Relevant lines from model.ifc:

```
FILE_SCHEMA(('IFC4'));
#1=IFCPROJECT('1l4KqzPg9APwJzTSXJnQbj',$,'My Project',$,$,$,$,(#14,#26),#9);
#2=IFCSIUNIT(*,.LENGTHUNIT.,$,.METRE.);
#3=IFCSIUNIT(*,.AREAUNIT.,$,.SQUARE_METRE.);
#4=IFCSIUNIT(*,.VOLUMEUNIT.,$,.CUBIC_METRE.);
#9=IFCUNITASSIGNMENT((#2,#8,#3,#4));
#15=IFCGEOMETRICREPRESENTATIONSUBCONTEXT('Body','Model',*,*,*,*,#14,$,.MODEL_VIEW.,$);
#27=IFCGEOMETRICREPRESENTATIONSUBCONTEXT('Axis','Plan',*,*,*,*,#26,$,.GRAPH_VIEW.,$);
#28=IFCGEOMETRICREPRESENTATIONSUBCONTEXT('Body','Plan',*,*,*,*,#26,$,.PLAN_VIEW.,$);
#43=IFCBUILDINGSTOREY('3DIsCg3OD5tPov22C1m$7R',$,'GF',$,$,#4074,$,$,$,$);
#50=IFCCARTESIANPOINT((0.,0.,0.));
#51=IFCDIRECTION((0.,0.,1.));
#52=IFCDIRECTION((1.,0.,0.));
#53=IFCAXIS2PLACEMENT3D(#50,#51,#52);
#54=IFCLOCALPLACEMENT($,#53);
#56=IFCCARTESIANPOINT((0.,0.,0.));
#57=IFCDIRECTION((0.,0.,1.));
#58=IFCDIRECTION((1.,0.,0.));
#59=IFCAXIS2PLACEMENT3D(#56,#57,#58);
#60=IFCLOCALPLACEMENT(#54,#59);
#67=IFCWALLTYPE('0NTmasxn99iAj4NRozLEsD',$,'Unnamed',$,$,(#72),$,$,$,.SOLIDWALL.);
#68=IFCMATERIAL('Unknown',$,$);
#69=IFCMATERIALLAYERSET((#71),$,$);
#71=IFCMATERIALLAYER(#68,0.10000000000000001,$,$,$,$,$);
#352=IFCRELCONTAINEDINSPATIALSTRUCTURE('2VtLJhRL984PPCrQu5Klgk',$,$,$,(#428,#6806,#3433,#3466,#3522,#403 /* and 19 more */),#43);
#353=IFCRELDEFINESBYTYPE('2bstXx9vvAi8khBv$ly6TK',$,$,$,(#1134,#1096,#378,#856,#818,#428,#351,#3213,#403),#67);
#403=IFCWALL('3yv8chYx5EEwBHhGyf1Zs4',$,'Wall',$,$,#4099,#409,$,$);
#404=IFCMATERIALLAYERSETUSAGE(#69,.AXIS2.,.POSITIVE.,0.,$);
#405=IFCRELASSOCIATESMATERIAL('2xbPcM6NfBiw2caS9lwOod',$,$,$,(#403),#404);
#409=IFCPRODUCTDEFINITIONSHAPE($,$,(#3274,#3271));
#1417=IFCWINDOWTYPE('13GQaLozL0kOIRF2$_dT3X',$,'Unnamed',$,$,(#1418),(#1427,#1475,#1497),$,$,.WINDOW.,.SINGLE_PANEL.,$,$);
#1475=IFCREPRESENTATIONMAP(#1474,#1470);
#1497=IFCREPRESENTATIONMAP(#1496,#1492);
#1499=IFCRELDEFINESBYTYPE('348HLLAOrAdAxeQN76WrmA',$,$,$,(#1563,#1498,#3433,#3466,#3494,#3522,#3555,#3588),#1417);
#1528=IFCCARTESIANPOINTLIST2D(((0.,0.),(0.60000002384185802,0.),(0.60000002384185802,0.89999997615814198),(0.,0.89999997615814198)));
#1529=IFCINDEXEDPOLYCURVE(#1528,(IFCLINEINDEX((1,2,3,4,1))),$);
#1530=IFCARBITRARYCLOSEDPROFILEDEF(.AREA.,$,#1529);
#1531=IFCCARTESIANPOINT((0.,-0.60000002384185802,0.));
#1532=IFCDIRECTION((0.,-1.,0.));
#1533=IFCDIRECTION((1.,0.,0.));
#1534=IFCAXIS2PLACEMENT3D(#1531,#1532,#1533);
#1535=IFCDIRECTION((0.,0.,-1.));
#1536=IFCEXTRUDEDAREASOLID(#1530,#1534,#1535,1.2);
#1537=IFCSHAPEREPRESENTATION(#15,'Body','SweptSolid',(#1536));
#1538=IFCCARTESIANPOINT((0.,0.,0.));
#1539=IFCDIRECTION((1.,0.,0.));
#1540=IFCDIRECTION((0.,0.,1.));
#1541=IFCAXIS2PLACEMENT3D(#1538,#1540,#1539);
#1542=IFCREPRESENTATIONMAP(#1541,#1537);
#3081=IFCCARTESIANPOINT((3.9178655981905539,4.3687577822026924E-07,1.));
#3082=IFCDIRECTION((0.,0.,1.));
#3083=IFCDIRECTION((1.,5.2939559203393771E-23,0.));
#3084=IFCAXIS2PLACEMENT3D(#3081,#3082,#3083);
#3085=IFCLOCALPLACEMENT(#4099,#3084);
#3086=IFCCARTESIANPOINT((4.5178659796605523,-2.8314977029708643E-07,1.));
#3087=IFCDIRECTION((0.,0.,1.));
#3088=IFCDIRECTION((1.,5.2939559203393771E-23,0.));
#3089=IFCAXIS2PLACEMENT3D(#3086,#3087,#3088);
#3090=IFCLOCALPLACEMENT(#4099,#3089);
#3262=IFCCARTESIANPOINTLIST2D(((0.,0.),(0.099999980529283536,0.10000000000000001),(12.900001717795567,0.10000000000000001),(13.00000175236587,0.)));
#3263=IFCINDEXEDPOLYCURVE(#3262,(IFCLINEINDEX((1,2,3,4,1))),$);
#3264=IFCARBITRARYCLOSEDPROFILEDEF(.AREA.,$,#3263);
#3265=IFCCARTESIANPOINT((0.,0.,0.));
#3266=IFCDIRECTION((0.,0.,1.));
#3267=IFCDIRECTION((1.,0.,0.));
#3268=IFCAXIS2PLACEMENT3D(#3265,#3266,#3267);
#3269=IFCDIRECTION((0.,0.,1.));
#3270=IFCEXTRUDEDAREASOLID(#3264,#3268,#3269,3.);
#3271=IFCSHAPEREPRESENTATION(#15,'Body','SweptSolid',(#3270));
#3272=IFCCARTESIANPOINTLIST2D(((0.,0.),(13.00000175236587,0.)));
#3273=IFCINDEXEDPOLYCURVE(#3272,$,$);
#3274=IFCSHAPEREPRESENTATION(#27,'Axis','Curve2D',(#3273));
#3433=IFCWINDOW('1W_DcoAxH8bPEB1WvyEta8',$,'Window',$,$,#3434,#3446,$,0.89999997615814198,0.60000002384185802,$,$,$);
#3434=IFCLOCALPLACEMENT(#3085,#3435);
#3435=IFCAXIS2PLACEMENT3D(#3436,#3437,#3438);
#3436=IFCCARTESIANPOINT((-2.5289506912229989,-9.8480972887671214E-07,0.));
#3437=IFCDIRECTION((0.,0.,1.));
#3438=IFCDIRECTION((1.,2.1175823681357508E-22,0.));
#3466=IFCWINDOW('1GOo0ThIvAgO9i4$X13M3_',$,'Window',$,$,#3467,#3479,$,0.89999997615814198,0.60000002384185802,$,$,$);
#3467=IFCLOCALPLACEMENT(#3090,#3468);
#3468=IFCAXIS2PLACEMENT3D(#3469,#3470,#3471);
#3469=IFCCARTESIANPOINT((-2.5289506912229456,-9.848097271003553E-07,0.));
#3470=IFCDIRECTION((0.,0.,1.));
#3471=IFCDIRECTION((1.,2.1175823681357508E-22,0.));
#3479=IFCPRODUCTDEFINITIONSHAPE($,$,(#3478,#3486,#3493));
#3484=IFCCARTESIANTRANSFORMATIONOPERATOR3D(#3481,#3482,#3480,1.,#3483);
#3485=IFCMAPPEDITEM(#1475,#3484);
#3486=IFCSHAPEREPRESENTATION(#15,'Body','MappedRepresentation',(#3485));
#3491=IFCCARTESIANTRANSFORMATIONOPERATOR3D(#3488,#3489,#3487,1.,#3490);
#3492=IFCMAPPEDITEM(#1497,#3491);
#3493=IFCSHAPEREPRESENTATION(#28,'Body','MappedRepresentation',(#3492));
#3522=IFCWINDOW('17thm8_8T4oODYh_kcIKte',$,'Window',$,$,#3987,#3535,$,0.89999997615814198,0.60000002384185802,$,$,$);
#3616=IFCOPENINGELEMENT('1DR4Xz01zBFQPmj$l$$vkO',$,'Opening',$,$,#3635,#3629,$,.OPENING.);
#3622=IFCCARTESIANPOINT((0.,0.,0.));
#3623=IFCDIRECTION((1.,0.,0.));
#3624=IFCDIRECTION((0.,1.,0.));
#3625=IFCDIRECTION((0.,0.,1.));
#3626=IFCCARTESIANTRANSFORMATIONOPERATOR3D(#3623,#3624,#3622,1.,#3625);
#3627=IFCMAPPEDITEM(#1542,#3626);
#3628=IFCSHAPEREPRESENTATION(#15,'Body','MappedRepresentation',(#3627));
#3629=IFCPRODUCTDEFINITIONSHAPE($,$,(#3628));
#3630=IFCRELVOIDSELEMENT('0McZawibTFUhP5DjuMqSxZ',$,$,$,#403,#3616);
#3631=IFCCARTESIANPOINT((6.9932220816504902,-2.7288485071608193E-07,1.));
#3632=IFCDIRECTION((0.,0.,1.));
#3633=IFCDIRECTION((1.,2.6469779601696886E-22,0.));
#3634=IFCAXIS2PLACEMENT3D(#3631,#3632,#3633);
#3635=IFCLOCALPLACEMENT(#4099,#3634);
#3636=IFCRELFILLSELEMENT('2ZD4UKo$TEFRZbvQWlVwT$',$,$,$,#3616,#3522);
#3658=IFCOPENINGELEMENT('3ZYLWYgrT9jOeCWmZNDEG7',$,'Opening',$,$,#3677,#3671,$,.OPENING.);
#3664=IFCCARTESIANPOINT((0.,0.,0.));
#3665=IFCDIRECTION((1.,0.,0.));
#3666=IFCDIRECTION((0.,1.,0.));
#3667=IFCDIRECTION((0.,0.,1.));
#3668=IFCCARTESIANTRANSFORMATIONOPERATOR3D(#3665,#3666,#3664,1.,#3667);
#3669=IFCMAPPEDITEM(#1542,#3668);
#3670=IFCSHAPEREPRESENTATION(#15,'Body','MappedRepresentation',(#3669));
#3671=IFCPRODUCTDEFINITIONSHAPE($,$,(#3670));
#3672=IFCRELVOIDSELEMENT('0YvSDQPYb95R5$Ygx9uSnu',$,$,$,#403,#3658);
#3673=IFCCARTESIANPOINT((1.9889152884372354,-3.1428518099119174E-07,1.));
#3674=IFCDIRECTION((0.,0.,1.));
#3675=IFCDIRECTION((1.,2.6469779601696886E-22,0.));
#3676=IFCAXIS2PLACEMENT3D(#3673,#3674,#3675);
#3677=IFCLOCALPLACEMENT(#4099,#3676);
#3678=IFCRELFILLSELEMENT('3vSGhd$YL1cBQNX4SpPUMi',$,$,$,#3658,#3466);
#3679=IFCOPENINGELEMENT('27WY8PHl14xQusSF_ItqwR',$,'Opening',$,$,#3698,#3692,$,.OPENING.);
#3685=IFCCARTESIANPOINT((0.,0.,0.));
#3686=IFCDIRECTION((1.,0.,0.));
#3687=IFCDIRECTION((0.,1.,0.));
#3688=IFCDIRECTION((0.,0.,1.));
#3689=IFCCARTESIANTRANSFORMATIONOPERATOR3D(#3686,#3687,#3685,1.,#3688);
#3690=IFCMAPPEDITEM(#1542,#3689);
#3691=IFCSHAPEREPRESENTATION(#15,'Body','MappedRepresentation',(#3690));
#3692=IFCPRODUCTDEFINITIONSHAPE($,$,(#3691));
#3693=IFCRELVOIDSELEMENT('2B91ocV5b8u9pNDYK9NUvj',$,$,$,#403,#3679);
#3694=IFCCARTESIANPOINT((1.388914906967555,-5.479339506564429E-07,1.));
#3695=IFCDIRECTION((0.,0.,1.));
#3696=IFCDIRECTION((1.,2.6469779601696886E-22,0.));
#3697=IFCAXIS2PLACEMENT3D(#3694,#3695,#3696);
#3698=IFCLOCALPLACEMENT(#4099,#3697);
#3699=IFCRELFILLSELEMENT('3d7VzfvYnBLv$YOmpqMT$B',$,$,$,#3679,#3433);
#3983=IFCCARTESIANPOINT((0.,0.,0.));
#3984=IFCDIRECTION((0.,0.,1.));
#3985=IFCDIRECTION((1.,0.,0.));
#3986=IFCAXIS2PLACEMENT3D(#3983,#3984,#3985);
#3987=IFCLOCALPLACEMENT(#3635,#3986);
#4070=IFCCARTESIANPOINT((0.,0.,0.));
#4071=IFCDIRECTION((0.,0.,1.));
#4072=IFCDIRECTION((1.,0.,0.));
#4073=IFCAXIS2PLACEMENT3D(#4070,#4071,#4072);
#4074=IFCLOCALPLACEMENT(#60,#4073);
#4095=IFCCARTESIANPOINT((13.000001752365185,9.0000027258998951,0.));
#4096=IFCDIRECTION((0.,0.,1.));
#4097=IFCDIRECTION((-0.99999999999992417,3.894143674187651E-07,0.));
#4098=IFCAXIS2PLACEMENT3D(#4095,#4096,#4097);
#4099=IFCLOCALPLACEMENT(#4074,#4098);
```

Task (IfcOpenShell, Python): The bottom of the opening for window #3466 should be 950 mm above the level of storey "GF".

```python
import numpy as np
import ifcopenshell
import ifcopenshell.api.geometry
import ifcopenshell.geom
import ifcopenshell.util.element
import ifcopenshell.util.placement
import ifcopenshell.util.shape
import ifcopenshell.util.unit

model = ifcopenshell.open("model.ifc")
unit_scale = ifcopenshell.util.unit.calculate_unit_scale(model)

window = model.by_guid("1GOo0ThIvAgO9i4$X13M3_")
opening = window.FillsVoids[0].RelatingOpeningElement
storey = ifcopenshell.util.element.get_container(window, ifc_class="IfcBuildingStorey")
level = ifcopenshell.util.placement.get_local_placement(storey.ObjectPlacement)[2, 3]

# The opening's origin need not be at the sill, so measure its lowest point.
shape = ifcopenshell.geom.create_shape(ifcopenshell.geom.settings(), opening)
bottom = ifcopenshell.util.shape.get_shape_bottom_elevation(shape, shape.geometry) / unit_scale
dz = level + 0.95 - bottom

shift = np.array([0.0, 0.0, dz])
# The window is not placed relative to its opening, so move both.
for product in (opening, window):
    matrix = ifcopenshell.util.placement.get_local_placement(product.ObjectPlacement)
    matrix[:3, 3] += shift
    ifcopenshell.api.geometry.edit_object_placement(model, product=product, matrix=matrix, is_si=False)

print(f"moved by {dz * unit_scale:+.3f} m")

model.write("model_v2.ifc")
```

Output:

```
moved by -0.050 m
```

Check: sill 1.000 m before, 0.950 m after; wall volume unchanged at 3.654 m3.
